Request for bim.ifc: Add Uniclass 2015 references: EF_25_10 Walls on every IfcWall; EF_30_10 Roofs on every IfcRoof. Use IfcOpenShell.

First a look at what the model holds.

```python
import ifcopenshell

model = ifcopenshell.open("bim.ifc")
print(model.schema)
print("classifications:", [c.Name for c in model.by_type("IfcClassification")])
for ifc_class in ("IfcDoor", "IfcRoof", "IfcStair", "IfcWall", "IfcWindow"):
    print(ifc_class, len(model.by_type(ifc_class)))
```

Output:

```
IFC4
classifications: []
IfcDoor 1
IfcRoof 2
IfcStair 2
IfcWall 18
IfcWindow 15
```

```python
import ifcopenshell
import ifcopenshell.api.classification

model = ifcopenshell.open("bim.ifc")

system = ifcopenshell.api.classification.add_classification(model, classification="Uniclass 2015")

codes = {
    "IfcWall": ("EF_25_10", "Walls"),
    "IfcRoof": ("EF_30_10", "Roofs"),
}
for ifc_class, (code, name) in codes.items():
    products = model.by_type(ifc_class)
    ifcopenshell.api.classification.add_reference(
        model, products=products, classification=system, identification=code, name=name
    )
    print(code, len(products))

model.write("bim_rev.ifc")
```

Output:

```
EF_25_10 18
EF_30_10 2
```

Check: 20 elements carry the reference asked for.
